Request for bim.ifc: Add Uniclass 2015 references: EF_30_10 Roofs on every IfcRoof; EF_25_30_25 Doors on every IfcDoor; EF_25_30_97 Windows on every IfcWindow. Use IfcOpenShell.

First a look at what the model holds.

```python
import ifcopenshell

model = ifcopenshell.open("bim.ifc")
print(model.schema)
print("classifications:", [c.Name for c in model.by_type("IfcClassification")])
for ifc_class in ("IfcDoor", "IfcRoof", "IfcStair", "IfcWall", "IfcWindow"):
    print(ifc_class, len(model.by_type(ifc_class)))
```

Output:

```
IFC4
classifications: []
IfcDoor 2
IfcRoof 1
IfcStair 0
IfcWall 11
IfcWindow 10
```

```python
import ifcopenshell
import ifcopenshell.api.classification

model = ifcopenshell.open("bim.ifc")

system = ifcopenshell.api.classification.add_classification(model, classification="Uniclass 2015")

codes = {
    "IfcRoof": ("EF_30_10", "Roofs"),
    "IfcDoor": ("EF_25_30_25", "Doors"),
    "IfcWindow": ("EF_25_30_97", "Windows"),
}
for ifc_class, (code, name) in codes.items():
    products = model.by_type(ifc_class)
    ifcopenshell.api.classification.add_reference(
        model, products=products, classification=system, identification=code, name=name
    )
    print(code, len(products))

model.write("bim_v2.ifc")
```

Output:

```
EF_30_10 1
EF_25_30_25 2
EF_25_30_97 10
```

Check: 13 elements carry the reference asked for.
